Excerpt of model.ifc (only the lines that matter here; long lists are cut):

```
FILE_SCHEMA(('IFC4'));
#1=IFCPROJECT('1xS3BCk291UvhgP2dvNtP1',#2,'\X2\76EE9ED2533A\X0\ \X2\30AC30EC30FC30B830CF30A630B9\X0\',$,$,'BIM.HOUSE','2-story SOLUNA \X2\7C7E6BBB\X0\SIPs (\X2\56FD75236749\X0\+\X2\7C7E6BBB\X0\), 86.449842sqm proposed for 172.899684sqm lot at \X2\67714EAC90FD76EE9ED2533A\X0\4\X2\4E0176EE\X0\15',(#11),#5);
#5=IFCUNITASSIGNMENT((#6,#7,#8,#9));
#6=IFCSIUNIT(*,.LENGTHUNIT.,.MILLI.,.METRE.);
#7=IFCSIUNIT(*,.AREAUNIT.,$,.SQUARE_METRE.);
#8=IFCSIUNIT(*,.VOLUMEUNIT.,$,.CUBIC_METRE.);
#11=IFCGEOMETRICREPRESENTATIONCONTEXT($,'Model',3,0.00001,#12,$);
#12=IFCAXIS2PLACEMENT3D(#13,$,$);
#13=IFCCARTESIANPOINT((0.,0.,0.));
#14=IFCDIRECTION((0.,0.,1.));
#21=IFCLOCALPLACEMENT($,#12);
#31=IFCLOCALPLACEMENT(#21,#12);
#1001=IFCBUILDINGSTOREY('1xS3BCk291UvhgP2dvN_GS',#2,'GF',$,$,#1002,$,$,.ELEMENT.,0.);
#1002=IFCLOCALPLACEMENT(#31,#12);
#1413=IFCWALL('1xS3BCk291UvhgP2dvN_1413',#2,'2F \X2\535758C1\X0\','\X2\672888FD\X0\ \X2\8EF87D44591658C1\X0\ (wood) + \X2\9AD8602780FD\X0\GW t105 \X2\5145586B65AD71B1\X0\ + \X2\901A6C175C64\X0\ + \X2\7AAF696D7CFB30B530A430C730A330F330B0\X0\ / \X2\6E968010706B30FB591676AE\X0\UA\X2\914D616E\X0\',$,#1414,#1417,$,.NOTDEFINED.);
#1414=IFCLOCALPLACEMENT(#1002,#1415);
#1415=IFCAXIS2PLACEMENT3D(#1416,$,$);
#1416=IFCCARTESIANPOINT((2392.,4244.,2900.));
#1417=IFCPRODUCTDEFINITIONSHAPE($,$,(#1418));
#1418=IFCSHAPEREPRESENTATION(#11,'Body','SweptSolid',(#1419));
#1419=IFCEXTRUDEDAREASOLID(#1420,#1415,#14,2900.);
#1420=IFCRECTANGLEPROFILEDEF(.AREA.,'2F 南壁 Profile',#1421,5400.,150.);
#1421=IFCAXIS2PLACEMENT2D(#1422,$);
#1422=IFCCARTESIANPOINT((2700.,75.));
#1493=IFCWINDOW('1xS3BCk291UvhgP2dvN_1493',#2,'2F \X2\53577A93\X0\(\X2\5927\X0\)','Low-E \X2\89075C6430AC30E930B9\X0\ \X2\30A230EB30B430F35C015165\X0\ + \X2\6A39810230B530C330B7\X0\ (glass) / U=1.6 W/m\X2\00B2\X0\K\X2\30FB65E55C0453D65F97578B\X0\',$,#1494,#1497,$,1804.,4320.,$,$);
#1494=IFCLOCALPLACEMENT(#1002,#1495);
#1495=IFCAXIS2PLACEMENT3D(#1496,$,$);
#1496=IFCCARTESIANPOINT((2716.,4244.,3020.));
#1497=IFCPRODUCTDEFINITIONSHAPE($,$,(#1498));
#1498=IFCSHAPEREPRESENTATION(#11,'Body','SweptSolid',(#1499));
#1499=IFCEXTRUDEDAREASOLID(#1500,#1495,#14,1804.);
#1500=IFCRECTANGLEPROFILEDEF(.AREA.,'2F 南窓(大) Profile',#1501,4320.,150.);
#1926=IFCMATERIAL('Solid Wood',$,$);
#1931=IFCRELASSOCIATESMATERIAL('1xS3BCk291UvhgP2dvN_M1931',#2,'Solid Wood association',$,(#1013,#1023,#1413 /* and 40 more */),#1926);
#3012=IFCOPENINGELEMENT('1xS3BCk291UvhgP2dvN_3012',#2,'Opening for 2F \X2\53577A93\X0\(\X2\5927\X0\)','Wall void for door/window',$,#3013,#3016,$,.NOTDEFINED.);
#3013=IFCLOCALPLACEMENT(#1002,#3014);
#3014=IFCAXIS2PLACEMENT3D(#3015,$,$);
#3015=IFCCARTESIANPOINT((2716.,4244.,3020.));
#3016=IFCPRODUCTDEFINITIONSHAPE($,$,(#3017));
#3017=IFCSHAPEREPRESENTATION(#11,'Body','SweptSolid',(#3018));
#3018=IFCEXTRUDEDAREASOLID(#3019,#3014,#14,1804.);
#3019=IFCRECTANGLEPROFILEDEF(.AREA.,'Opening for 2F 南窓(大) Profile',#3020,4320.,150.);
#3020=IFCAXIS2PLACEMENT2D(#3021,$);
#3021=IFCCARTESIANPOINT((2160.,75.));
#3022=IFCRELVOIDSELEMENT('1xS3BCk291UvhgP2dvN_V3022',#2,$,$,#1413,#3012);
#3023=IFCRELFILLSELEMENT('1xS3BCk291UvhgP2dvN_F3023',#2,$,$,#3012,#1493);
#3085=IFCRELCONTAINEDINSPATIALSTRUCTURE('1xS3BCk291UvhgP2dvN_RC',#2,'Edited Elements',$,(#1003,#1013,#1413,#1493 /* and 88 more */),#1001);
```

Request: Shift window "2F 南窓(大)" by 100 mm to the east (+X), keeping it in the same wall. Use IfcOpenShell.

```python
import ifcopenshell
import ifcopenshell.api.geometry
import ifcopenshell.util.placement
import ifcopenshell.util.unit

model = ifcopenshell.open("model.ifc")
unit_scale = ifcopenshell.util.unit.calculate_unit_scale(model)

window = model.by_guid("1xS3BCk291UvhgP2dvN_1493")
opening = window.FillsVoids[0].RelatingOpeningElement
wall = opening.VoidsElements[0].RelatingBuildingElement

wall_matrix = ifcopenshell.util.placement.get_local_placement(wall.ObjectPlacement)
shift = wall_matrix[:3, 0] * 0.1 / unit_scale
before = ifcopenshell.util.placement.get_local_placement(window.ObjectPlacement)[:3, 3].copy()

# The window is not placed relative to its opening, so move both.
for product in (opening, window):
    matrix = ifcopenshell.util.placement.get_local_placement(product.ObjectPlacement)
    matrix[:3, 3] += shift
    ifcopenshell.api.geometry.edit_object_placement(model, product=product, matrix=matrix, is_si=False)

after = ifcopenshell.util.placement.get_local_placement(window.ObjectPlacement)[:3, 3]
print("window moved by", (after - before).round(3) + 0.0)

model.write("model-out.ifc")
```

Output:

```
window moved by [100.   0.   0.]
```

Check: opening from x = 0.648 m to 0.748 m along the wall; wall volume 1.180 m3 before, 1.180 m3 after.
